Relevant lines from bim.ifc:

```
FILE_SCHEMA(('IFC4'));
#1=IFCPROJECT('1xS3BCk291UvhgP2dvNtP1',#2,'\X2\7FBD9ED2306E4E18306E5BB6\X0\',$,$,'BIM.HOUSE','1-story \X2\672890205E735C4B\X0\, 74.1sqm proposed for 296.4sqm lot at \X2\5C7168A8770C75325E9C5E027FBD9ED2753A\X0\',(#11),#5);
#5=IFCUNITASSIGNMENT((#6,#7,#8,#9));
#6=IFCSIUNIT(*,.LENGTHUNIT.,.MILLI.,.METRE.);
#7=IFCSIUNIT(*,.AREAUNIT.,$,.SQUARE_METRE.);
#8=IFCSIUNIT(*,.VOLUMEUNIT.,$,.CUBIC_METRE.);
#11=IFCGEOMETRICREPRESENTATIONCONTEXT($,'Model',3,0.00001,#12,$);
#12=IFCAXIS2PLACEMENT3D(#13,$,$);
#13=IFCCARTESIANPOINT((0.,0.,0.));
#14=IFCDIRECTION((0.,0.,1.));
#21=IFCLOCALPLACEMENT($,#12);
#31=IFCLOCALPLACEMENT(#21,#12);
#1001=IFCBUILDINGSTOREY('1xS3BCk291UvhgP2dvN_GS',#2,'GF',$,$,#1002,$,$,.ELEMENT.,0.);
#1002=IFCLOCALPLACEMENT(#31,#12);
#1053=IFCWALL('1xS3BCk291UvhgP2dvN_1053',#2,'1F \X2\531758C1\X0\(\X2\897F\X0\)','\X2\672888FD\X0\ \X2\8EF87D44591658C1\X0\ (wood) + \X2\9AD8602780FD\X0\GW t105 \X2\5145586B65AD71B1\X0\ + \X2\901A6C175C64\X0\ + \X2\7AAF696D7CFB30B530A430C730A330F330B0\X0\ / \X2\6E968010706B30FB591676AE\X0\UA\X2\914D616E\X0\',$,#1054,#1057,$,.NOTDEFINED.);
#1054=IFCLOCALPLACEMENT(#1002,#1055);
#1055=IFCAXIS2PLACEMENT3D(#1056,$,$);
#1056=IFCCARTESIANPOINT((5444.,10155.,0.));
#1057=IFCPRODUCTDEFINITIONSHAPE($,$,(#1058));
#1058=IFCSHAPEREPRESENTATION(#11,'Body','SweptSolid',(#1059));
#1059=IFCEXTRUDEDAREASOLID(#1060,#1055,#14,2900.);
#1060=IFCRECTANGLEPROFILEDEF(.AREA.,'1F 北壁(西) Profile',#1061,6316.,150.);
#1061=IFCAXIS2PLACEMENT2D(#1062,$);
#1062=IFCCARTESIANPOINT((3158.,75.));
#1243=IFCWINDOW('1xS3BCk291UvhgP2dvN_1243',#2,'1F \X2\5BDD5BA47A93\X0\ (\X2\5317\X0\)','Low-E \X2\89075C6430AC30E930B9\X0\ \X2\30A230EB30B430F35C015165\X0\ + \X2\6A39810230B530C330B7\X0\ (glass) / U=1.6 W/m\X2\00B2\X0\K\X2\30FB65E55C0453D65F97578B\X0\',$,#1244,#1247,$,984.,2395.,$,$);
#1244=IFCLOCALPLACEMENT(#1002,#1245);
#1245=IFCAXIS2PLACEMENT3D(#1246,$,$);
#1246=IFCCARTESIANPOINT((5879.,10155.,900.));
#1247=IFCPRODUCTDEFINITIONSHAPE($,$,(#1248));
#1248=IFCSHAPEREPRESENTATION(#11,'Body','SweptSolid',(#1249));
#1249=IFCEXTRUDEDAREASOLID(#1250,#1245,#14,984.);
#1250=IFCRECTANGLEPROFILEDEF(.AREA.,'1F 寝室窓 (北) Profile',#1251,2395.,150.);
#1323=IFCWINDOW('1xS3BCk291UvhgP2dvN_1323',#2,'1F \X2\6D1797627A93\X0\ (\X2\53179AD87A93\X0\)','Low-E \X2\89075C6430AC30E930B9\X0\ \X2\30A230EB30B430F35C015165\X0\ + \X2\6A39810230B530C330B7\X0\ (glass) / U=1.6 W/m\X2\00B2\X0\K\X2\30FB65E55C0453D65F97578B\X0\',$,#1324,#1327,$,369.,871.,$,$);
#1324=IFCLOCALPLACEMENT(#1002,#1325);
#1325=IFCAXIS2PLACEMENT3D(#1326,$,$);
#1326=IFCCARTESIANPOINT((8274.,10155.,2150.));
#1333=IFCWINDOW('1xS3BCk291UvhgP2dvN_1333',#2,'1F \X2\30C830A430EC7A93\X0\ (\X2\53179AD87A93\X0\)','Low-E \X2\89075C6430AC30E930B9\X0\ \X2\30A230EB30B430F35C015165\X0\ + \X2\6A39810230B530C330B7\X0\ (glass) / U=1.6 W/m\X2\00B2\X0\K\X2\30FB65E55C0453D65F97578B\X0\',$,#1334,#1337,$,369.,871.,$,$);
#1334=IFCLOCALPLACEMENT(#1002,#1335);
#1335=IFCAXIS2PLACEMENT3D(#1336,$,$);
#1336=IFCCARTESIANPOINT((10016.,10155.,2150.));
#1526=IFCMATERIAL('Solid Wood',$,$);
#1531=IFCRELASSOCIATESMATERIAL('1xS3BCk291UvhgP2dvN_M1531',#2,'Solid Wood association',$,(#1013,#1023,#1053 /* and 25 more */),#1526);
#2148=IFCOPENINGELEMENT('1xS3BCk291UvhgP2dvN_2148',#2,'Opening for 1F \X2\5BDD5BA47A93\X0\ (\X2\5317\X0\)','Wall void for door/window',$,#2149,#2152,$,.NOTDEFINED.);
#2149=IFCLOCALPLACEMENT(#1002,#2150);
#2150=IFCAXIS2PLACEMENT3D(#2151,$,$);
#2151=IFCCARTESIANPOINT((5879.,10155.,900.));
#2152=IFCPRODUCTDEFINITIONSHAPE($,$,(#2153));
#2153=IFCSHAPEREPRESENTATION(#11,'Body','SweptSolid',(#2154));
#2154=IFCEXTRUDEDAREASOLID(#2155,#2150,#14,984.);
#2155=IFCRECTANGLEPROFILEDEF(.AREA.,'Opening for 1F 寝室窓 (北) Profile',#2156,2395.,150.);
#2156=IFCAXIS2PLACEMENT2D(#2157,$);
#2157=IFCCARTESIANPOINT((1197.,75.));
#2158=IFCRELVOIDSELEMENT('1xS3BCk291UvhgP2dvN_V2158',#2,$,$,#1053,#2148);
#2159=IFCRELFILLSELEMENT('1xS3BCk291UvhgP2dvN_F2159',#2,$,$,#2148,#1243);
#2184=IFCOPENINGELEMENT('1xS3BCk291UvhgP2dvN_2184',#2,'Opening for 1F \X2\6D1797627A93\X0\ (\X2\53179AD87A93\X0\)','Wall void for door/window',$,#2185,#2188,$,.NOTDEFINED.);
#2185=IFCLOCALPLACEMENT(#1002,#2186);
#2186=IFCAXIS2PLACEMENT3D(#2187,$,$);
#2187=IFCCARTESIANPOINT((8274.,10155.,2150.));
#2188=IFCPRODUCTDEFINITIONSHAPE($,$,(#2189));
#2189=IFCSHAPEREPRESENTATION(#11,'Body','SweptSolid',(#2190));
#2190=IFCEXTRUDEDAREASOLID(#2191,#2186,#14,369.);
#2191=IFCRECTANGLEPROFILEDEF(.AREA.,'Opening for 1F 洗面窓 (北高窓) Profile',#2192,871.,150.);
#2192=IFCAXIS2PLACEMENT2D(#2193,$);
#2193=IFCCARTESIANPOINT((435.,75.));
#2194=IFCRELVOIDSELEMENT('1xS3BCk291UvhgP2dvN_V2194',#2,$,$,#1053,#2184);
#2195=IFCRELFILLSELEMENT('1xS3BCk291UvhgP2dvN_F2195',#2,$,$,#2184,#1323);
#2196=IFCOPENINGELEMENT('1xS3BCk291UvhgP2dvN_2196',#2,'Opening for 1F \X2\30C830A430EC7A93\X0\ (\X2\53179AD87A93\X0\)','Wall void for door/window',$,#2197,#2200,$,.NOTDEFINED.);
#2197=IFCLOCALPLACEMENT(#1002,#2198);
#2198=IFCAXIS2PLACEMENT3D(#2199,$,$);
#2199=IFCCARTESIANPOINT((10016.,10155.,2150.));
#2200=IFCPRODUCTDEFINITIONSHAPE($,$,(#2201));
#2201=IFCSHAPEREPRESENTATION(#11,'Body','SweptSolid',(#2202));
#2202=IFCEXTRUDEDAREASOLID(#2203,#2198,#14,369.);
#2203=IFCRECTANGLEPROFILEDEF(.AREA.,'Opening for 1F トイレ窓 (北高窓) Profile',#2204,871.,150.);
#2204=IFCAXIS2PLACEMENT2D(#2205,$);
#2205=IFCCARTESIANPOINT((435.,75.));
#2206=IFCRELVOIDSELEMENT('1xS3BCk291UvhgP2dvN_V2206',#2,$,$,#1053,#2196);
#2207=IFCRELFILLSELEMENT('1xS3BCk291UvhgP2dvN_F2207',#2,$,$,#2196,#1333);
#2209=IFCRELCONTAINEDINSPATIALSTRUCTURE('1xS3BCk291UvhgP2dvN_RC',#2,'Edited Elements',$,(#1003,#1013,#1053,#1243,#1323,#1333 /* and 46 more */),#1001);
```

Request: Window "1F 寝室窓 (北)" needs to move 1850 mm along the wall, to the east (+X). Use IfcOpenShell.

```python
import ifcopenshell
import ifcopenshell.api.geometry
import ifcopenshell.util.placement
import ifcopenshell.util.unit

model = ifcopenshell.open("bim.ifc")
unit_scale = ifcopenshell.util.unit.calculate_unit_scale(model)

window = model.by_id(1243)
opening = window.FillsVoids[0].RelatingOpeningElement
wall = opening.VoidsElements[0].RelatingBuildingElement

wall_matrix = ifcopenshell.util.placement.get_local_placement(wall.ObjectPlacement)
shift = wall_matrix[:3, 0] * 1.85 / unit_scale
before = ifcopenshell.util.placement.get_local_placement(window.ObjectPlacement)[:3, 3].copy()

# The window is not placed relative to its opening, so move both.
for product in (opening, window):
    matrix = ifcopenshell.util.placement.get_local_placement(product.ObjectPlacement)
    matrix[:3, 3] += shift
    ifcopenshell.api.geometry.edit_object_placement(model, product=product, matrix=matrix, is_si=False)

after = ifcopenshell.util.placement.get_local_placement(window.ObjectPlacement)[:3, 3]
print("window moved by", (after - before).round(3) + 0.0)

model.write("bim_rev.ifc")
```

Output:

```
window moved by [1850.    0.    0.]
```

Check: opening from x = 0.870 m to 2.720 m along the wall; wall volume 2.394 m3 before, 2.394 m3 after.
